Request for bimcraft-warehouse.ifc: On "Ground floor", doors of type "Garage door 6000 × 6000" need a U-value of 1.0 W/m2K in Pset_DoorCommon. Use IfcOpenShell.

First a look at what the model holds.

```python
import ifcopenshell
import ifcopenshell.util.element

model = ifcopenshell.open("bimcraft-warehouse.ifc")
print(model.schema)
storey = next(s for s in model.by_type("IfcBuildingStorey") if s.Name == "Ground floor")
doors = [e for e in ifcopenshell.util.element.get_decomposition(storey) if e.is_a("IfcDoor")]
seen = {}
for e in doors:
    element_type = ifcopenshell.util.element.get_type(e)
    key = (element_type.Name if element_type != e and element_type else None, ifcopenshell.util.element.get_pset(e, "Pset_DoorCommon", "ThermalTransmittance"))
    seen[key] = seen.get(key, 0) + 1
for (name, value), count in sorted(seen.items(), key=str):
    print(count, "x", name, "|", value)
```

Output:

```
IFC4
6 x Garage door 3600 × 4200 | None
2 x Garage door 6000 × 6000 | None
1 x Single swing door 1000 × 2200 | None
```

```python
import ifcopenshell
import ifcopenshell.api.pset
import ifcopenshell.util.element

model = ifcopenshell.open("bimcraft-warehouse.ifc")

storey = next(s for s in model.by_type("IfcBuildingStorey") if s.Name == "Ground floor")
doors = [e for e in ifcopenshell.util.element.get_decomposition(storey) if e.is_a("IfcDoor")]

count = 0
for e in doors:
    element_type = ifcopenshell.util.element.get_type(e)
    if element_type in (None, e) or element_type.Name != "Garage door 6000 × 6000":
        continue
    # add_pset returns the element's existing set when there is one.
    pset = ifcopenshell.api.pset.add_pset(model, product=e, name="Pset_DoorCommon")
    ifcopenshell.api.pset.edit_pset(model, pset=pset, properties={"ThermalTransmittance": 1.0})
    count += 1

print(count, "doors updated")

model.write("bimcraft-warehouse_edited.ifc")
```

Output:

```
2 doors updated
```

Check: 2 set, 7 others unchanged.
